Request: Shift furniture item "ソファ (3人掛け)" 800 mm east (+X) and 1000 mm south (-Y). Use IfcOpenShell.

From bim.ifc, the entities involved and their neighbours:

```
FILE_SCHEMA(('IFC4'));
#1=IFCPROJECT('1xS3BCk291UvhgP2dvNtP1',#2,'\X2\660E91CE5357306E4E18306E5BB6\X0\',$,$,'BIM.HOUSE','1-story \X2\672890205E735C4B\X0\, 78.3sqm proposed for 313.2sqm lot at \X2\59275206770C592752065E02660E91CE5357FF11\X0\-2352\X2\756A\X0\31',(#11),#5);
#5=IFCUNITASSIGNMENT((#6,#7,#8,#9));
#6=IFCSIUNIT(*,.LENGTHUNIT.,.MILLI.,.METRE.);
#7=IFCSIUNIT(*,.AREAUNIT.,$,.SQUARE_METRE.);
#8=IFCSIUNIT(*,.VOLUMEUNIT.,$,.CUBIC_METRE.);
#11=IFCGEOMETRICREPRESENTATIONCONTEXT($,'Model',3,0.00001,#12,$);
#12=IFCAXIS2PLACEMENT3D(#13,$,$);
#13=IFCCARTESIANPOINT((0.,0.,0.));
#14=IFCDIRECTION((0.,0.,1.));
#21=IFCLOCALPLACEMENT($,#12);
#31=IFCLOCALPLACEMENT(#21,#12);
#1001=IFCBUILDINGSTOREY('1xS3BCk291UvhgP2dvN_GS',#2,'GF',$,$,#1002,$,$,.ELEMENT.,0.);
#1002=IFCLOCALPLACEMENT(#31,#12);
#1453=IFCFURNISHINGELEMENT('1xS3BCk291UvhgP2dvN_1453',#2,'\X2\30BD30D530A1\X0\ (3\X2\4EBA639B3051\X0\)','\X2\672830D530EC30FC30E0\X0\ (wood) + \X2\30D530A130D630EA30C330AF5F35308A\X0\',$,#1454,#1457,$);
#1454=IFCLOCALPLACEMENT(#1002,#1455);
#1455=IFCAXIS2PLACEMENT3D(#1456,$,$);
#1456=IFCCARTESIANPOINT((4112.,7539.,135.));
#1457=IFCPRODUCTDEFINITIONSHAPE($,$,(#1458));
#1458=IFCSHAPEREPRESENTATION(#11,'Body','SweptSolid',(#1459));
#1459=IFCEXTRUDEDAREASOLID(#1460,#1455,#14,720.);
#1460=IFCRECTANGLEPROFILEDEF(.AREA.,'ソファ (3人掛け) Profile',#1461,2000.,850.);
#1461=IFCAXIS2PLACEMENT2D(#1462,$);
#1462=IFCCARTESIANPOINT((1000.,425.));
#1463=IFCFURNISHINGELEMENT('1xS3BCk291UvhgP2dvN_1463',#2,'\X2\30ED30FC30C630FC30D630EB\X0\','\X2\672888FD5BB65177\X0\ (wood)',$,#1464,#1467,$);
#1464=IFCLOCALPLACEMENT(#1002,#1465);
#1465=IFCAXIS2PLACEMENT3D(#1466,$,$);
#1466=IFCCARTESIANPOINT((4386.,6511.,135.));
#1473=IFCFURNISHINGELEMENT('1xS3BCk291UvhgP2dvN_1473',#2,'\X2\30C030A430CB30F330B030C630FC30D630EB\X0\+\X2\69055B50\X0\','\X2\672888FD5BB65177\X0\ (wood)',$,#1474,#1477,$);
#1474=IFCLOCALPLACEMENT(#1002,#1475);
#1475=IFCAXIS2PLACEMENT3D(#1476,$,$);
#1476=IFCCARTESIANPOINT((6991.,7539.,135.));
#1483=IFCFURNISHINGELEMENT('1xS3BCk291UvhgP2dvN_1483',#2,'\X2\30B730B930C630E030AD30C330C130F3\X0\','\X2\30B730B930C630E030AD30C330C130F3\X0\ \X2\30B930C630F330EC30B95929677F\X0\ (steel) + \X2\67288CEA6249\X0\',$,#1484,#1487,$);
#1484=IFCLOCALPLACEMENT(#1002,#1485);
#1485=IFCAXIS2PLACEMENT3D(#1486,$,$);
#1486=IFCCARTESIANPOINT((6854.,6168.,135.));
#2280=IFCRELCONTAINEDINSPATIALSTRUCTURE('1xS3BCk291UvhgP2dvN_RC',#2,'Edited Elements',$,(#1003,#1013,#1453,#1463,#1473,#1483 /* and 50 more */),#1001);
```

```python
import ifcopenshell
import ifcopenshell.api.geometry
import ifcopenshell.util.placement

model = ifcopenshell.open("bim.ifc")

item = model.by_guid("1xS3BCk291UvhgP2dvN_1453")
matrix = ifcopenshell.util.placement.get_local_placement(item.ObjectPlacement)
matrix[0, 3] += 800.0
matrix[1, 3] -= 1000.0
ifcopenshell.api.geometry.edit_object_placement(model, product=item, matrix=matrix, is_si=False)

print(ifcopenshell.util.placement.get_local_placement(item.ObjectPlacement).round(3) + 0.0)

model.write("bim_updated.ifc")
```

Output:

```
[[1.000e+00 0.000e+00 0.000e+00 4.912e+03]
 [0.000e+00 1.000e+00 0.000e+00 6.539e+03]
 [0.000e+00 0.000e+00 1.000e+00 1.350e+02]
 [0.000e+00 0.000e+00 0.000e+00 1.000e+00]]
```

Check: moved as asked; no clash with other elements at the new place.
